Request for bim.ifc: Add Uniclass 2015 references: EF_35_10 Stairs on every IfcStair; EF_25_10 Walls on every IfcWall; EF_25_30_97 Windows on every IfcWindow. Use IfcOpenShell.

First a look at what the model holds.

```python
import ifcopenshell

model = ifcopenshell.open("bim.ifc")
print(model.schema)
print("classifications:", [c.Name for c in model.by_type("IfcClassification")])
for ifc_class in ("IfcDoor", "IfcRoof", "IfcStair", "IfcWall", "IfcWindow"):
    print(ifc_class, len(model.by_type(ifc_class)))
```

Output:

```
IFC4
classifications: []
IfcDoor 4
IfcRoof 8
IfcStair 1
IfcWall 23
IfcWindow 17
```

```python
import ifcopenshell
import ifcopenshell.api.classification

model = ifcopenshell.open("bim.ifc")

system = ifcopenshell.api.classification.add_classification(model, classification="Uniclass 2015")

codes = {
    "IfcStair": ("EF_35_10", "Stairs"),
    "IfcWall": ("EF_25_10", "Walls"),
    "IfcWindow": ("EF_25_30_97", "Windows"),
}
for ifc_class, (code, name) in codes.items():
    products = model.by_type(ifc_class)
    ifcopenshell.api.classification.add_reference(
        model, products=products, classification=system, identification=code, name=name
    )
    print(code, len(products))

model.write("bim_rev.ifc")
```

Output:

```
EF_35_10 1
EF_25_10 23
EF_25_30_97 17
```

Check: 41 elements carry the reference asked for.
